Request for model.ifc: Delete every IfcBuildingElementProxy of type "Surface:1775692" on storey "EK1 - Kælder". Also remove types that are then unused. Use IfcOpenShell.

First a look at what the model holds.

```python
import ifcopenshell
import ifcopenshell.util.element

model = ifcopenshell.open("model.ifc")
print(model.schema)
storey = next(s for s in model.by_type("IfcBuildingStorey") if s.Name == "EK1 - Kælder")
proxies = [e for e in ifcopenshell.util.element.get_decomposition(storey) if e.is_a("IfcBuildingElementProxy")]
seen = {}
for e in proxies:
    element_type = ifcopenshell.util.element.get_type(e)
    name = element_type.Name if element_type not in (None, e) else None
    seen[name] = seen.get(name, 0) + 1
for name, count in sorted(seen.items(), key=str):
    print(count, "x", name)
```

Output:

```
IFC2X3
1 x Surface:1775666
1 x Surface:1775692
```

```python
import ifcopenshell
import ifcopenshell.api.root
import ifcopenshell.util.element

model = ifcopenshell.open("model.ifc")

storey = next(s for s in model.by_type("IfcBuildingStorey") if s.Name == "EK1 - Kælder")
proxies = [e for e in ifcopenshell.util.element.get_decomposition(storey) if e.is_a("IfcBuildingElementProxy")]
targets = [e for e in proxies if (t := ifcopenshell.util.element.get_type(e)) not in (None, e) and t.Name == "Surface:1775692"]
types = {ifcopenshell.util.element.get_type(e) for e in targets} - {None, *targets}

for e in targets:
    ifcopenshell.api.root.remove_product(model, product=e)
print(len(targets), "removed")

unused = [t for t in types if not ifcopenshell.util.element.get_types(t)]
for t in unused:
    ifcopenshell.api.root.remove_product(model, product=t)
print(len(unused), "unused types removed")

model.write("model_updated.ifc")
```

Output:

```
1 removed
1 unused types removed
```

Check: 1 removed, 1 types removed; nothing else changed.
